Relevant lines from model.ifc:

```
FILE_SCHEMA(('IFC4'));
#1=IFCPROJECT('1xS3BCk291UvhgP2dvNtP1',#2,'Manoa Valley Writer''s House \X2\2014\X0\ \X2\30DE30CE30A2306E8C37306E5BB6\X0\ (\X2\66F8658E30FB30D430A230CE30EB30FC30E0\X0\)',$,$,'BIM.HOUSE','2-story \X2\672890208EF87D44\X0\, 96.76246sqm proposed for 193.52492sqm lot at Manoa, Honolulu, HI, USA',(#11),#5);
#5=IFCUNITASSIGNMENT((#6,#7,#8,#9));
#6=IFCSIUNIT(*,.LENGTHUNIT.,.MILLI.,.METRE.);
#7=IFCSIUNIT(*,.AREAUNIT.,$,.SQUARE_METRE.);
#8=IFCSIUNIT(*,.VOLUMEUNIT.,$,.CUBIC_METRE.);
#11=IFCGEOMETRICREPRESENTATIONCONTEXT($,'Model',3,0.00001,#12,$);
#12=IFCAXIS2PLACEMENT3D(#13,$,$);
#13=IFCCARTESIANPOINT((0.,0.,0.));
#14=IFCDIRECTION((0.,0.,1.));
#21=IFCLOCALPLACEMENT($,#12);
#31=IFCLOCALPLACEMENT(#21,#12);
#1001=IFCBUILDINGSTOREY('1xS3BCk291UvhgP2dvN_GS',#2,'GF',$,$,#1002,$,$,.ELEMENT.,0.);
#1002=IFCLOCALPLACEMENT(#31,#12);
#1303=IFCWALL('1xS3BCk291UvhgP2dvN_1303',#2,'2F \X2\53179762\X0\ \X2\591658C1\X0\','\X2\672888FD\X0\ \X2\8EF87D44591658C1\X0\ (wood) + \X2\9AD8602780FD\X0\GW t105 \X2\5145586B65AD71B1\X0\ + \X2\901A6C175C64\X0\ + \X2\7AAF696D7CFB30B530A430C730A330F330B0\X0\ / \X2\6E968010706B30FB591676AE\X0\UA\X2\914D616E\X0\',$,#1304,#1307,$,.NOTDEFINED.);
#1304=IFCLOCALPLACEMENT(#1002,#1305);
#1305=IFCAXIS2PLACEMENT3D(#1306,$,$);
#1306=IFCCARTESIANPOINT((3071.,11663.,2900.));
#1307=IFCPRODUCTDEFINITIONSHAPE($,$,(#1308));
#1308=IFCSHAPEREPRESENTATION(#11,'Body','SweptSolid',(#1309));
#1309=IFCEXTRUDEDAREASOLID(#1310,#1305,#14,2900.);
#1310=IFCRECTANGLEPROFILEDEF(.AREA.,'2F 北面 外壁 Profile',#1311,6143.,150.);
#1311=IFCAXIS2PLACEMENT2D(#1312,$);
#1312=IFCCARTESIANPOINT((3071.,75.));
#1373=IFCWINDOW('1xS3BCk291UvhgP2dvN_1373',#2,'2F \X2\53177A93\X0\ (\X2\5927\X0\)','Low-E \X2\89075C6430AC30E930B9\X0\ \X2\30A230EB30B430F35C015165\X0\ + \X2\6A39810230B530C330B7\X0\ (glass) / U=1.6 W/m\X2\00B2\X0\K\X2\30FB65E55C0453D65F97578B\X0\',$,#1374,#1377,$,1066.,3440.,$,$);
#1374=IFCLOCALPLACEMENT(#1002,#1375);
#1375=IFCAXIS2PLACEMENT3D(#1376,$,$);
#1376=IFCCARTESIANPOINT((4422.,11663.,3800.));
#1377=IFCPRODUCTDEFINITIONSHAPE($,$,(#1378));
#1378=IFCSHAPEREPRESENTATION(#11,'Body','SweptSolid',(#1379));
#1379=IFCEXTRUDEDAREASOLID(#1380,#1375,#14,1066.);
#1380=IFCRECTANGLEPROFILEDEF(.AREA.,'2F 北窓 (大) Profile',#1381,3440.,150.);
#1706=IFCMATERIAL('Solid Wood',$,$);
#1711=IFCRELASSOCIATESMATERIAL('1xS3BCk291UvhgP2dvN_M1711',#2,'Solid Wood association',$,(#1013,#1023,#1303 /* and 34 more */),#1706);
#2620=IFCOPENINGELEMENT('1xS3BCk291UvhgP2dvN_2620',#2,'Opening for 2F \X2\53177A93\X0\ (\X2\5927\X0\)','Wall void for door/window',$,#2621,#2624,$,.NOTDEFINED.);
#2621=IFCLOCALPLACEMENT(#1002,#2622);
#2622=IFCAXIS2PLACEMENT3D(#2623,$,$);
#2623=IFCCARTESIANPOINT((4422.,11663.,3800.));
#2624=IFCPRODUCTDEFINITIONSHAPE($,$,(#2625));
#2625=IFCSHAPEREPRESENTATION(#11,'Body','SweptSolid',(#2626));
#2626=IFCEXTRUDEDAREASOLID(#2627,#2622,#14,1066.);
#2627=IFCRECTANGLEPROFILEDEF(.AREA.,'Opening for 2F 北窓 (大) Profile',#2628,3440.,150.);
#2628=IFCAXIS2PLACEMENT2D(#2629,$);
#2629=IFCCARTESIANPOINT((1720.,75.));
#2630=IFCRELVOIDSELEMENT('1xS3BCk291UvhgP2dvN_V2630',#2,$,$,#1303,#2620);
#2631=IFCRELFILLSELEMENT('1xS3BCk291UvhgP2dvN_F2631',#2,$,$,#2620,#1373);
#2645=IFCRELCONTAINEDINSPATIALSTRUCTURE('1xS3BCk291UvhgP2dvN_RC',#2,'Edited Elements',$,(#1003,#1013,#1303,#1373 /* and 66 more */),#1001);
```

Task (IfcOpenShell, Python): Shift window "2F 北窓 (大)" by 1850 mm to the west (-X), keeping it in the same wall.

```python
import ifcopenshell
import ifcopenshell.api.geometry
import ifcopenshell.util.placement
import ifcopenshell.util.unit

model = ifcopenshell.open("model.ifc")
unit_scale = ifcopenshell.util.unit.calculate_unit_scale(model)

window = model.by_guid("1xS3BCk291UvhgP2dvN_1373")
opening = window.FillsVoids[0].RelatingOpeningElement
wall = opening.VoidsElements[0].RelatingBuildingElement

wall_matrix = ifcopenshell.util.placement.get_local_placement(wall.ObjectPlacement)
shift = wall_matrix[:3, 0] * -1.85 / unit_scale
before = ifcopenshell.util.placement.get_local_placement(window.ObjectPlacement)[:3, 3].copy()

# The window is not placed relative to its opening, so move both.
for product in (opening, window):
    matrix = ifcopenshell.util.placement.get_local_placement(product.ObjectPlacement)
    matrix[:3, 3] += shift
    ifcopenshell.api.geometry.edit_object_placement(model, product=product, matrix=matrix, is_si=False)

after = ifcopenshell.util.placement.get_local_placement(window.ObjectPlacement)[:3, 3]
print("window moved by", (after - before).round(3) + 0.0)

model.write("model_v2.ifc")
```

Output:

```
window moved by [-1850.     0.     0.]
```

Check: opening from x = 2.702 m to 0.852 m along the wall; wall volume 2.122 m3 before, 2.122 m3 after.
